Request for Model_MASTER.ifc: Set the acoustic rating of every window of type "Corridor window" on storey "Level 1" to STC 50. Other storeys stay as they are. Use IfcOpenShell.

First a look at what the model holds.

```python
import ifcopenshell
import ifcopenshell.util.element

model = ifcopenshell.open("Model_MASTER.ifc")
print(model.schema)
storey = next(s for s in model.by_type("IfcBuildingStorey") if s.Name == "Level 1")
windows = [e for e in ifcopenshell.util.element.get_decomposition(storey) if e.is_a("IfcWindow")]
seen = {}
for e in windows:
    element_type = ifcopenshell.util.element.get_type(e)
    key = (element_type.Name if element_type != e and element_type else None, ifcopenshell.util.element.get_pset(e, "Pset_WindowCommon", "AcousticRating"))
    seen[key] = seen.get(key, 0) + 1
for (name, value), count in sorted(seen.items(), key=str):
    print(count, "x", name, "|", value)
```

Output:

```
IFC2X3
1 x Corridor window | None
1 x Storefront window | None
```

```python
import ifcopenshell
import ifcopenshell.api.pset
import ifcopenshell.util.element

model = ifcopenshell.open("Model_MASTER.ifc")

storey = next(s for s in model.by_type("IfcBuildingStorey") if s.Name == "Level 1")
windows = [e for e in ifcopenshell.util.element.get_decomposition(storey) if e.is_a("IfcWindow")]

count = 0
for e in windows:
    element_type = ifcopenshell.util.element.get_type(e)
    if element_type in (None, e) or element_type.Name != "Corridor window":
        continue
    # add_pset returns the element's existing set when there is one.
    pset = ifcopenshell.api.pset.add_pset(model, product=e, name="Pset_WindowCommon")
    ifcopenshell.api.pset.edit_pset(model, pset=pset, properties={"AcousticRating": "STC 50"})
    count += 1

print(count, "windows updated")

model.write("Model_MASTER_updated.ifc")
```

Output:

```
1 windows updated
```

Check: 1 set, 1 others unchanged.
